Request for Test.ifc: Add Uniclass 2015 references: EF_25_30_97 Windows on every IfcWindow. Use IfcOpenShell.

First a look at what the model holds.

```python
import ifcopenshell

model = ifcopenshell.open("Test.ifc")
print(model.schema)
print("classifications:", [c.Name for c in model.by_type("IfcClassification")])
for ifc_class in ("IfcDoor", "IfcRoof", "IfcStair", "IfcWall", "IfcWindow"):
    print(ifc_class, len(model.by_type(ifc_class)))
```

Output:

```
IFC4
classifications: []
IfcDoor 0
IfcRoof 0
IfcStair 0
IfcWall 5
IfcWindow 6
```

```python
import ifcopenshell
import ifcopenshell.api.classification

model = ifcopenshell.open("Test.ifc")

system = ifcopenshell.api.classification.add_classification(model, classification="Uniclass 2015")

codes = {
    "IfcWindow": ("EF_25_30_97", "Windows"),
}
for ifc_class, (code, name) in codes.items():
    products = model.by_type(ifc_class)
    ifcopenshell.api.classification.add_reference(
        model, products=products, classification=system, identification=code, name=name
    )
    print(code, len(products))

model.write("Test_updated.ifc")
```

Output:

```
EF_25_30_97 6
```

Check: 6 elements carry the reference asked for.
